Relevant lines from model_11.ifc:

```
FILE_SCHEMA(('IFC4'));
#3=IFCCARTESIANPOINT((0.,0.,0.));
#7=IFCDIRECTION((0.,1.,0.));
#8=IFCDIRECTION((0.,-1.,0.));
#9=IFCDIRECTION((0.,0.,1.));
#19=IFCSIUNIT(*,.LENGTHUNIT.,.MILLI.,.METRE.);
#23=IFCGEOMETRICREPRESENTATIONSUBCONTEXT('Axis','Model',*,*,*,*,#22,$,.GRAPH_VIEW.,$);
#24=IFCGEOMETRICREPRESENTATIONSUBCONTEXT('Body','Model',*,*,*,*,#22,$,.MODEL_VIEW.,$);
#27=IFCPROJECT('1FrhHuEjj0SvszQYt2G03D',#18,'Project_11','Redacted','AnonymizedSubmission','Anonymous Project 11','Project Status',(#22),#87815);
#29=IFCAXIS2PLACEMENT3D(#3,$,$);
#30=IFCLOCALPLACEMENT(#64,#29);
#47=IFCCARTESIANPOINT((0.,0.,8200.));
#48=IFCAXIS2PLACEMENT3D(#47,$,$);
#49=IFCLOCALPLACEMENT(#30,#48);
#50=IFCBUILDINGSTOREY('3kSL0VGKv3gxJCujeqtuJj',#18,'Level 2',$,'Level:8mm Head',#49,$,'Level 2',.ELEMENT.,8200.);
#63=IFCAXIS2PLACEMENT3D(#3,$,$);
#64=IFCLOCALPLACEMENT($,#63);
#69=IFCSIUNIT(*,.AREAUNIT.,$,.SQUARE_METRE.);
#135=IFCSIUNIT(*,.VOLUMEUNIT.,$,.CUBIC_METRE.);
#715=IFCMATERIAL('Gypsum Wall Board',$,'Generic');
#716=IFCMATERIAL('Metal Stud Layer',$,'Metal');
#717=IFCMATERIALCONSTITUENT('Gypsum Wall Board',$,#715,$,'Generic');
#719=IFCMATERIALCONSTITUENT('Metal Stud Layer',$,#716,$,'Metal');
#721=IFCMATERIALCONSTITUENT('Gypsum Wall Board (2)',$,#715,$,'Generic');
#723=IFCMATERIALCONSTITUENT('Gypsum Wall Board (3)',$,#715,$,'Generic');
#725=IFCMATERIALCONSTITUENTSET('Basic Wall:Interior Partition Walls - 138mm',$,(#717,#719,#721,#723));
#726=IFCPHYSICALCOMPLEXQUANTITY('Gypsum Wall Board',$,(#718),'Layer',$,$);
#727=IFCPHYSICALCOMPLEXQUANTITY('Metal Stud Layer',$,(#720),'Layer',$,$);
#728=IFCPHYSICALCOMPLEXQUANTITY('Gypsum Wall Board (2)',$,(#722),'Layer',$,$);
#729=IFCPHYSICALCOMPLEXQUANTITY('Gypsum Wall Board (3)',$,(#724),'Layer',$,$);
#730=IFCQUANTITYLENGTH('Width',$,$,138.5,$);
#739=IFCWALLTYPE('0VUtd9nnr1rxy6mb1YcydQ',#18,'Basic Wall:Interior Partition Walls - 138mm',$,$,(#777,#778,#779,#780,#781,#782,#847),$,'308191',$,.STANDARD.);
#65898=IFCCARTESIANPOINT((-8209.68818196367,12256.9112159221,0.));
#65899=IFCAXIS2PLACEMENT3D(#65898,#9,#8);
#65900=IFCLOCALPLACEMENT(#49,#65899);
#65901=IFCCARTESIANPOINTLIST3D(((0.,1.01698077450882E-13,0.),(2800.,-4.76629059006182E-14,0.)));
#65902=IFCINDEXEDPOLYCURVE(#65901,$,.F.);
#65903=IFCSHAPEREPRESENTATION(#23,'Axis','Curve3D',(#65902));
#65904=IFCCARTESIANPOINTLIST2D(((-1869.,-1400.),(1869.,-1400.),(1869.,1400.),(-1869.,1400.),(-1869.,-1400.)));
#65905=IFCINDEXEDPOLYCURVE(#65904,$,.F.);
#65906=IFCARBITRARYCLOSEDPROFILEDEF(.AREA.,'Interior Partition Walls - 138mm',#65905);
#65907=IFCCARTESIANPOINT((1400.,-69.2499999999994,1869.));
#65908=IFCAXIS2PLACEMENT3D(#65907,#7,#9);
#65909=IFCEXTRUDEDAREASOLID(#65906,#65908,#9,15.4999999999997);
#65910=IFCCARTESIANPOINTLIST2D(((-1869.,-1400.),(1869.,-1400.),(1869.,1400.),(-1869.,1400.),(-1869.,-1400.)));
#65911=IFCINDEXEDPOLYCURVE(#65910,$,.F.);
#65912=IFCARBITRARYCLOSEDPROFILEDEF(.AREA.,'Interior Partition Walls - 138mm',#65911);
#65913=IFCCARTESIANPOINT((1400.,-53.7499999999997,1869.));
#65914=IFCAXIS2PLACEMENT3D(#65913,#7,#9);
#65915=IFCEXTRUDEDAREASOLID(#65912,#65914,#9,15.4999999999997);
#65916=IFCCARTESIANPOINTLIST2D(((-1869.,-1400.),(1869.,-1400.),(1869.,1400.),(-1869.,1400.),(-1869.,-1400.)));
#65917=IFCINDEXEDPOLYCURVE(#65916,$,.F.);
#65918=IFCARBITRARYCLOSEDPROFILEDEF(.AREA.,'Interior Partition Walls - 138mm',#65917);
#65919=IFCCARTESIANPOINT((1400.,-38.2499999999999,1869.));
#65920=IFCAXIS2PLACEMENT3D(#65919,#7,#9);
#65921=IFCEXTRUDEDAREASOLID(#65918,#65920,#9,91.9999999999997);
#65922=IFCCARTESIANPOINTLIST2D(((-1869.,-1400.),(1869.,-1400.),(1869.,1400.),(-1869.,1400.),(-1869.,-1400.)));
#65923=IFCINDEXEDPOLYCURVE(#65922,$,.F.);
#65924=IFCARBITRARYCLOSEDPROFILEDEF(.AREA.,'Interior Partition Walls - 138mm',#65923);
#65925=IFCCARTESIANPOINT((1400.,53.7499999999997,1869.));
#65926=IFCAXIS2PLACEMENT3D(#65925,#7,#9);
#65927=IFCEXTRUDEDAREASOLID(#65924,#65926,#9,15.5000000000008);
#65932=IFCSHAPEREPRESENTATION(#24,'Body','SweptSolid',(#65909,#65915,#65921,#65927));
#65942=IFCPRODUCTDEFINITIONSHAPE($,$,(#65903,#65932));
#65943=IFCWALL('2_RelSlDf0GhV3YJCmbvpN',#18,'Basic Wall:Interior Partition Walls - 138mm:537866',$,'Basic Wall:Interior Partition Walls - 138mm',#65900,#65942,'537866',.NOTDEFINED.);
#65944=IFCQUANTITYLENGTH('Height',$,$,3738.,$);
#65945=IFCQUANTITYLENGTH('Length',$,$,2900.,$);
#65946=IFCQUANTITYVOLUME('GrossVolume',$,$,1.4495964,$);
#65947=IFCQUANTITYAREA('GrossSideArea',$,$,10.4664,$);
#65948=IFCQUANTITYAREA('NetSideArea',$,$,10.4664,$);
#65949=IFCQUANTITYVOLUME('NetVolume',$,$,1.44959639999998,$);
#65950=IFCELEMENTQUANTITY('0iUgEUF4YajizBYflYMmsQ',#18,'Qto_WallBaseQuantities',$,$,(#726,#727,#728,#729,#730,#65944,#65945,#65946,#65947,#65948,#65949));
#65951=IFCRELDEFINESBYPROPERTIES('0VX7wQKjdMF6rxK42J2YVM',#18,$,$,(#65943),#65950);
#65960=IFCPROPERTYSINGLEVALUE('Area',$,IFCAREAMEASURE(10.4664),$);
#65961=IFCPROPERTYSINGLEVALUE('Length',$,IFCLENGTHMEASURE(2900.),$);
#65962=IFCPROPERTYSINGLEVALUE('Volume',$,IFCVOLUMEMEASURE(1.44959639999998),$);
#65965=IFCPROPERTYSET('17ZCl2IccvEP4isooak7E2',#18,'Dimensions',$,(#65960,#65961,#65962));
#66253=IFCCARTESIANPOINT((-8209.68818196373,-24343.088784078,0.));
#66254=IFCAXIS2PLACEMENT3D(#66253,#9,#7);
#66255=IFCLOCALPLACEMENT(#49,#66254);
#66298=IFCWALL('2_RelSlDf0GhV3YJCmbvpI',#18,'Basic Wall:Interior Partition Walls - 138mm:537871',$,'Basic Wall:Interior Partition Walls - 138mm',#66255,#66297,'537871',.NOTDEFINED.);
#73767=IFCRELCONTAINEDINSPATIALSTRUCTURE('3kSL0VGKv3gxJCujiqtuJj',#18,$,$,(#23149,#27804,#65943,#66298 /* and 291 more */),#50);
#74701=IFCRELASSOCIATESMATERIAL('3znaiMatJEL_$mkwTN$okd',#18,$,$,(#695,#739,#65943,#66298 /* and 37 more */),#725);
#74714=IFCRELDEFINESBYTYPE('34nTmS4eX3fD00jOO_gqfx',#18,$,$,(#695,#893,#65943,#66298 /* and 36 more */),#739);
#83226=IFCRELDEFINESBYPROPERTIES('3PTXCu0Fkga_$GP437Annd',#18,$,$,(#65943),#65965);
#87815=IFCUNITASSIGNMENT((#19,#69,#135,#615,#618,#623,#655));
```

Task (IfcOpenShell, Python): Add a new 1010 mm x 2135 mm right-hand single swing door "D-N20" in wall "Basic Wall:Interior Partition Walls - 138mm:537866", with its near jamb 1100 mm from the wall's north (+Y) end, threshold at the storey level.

```python
import numpy as np
import ifcopenshell
import ifcopenshell.api.feature
import ifcopenshell.api.geometry
import ifcopenshell.api.pset
import ifcopenshell.api.root
import ifcopenshell.api.spatial
import ifcopenshell.geom
import ifcopenshell.util.element
import ifcopenshell.util.placement
import ifcopenshell.util.representation
import ifcopenshell.util.shape
import ifcopenshell.util.unit

model = ifcopenshell.open("model_11.ifc")
unit_scale = ifcopenshell.util.unit.calculate_unit_scale(model)
area_scale = ifcopenshell.util.unit.calculate_unit_scale(model, "AREAUNIT")
volume_scale = ifcopenshell.util.unit.calculate_unit_scale(model, "VOLUMEUNIT")
settings = ifcopenshell.geom.settings()


def volume(element):
    """Net volume in cubic metres, openings subtracted."""
    shape = ifcopenshell.geom.create_shape(settings, element)
    return ifcopenshell.util.shape.get_volume(shape.geometry)


wall = model.by_guid("2_RelSlDf0GhV3YJCmbvpN")
storey = ifcopenshell.util.element.get_container(wall, ifc_class="IfcBuildingStorey")
context = ifcopenshell.util.representation.get_context(model, "Model", "Body", "MODEL_VIEW")
before = volume(wall)

width, height, from_end, sill = 1.01, 2.135, 1.1, 0.0  # metres

# The wall runs along its own X axis, and the end named is its -X end.
wall_shape = ifcopenshell.geom.create_shape(settings, wall)
x, y, z = ifcopenshell.util.shape.get_vertices(wall_shape.geometry).T
start = x.min() + from_end
face, thickness = float(y.min()), float(y.max() - y.min())
wall_matrix = ifcopenshell.util.placement.get_local_placement(wall.ObjectPlacement)
level = ifcopenshell.util.placement.get_local_placement(storey.ObjectPlacement)[2, 3]


def in_wall(x, y):
    """Placement at x, y metres in the wall's axes, at sill height."""
    matrix = wall_matrix.copy()
    matrix[:, 3] = wall_matrix @ np.array([x / unit_scale, y / unit_scale, 0.0, 1.0])
    matrix[2, 3] = level + sill / unit_scale
    return matrix


# Opening: a box that overshoots both wall faces by 50 mm.
opening = ifcopenshell.api.root.create_entity(model, ifc_class="IfcOpeningElement", predefined_type="OPENING")
box = ifcopenshell.api.geometry.add_wall_representation(
    model, context=context, length=width, height=height, thickness=thickness + 0.1
)
ifcopenshell.api.geometry.assign_representation(model, product=opening, representation=box)
ifcopenshell.api.geometry.edit_object_placement(model, product=opening, matrix=in_wall(start, face - 0.05), is_si=False)
ifcopenshell.api.feature.add_feature(model, feature=opening, element=wall)

door = ifcopenshell.api.root.create_entity(model, ifc_class="IfcDoor", name="D-N20", predefined_type="DOOR")
door.OverallWidth, door.OverallHeight = width / unit_scale, height / unit_scale
door.OperationType = "SINGLE_SWING_RIGHT"
body = ifcopenshell.api.geometry.add_door_representation(
    model,
    context=context,
    overall_width=door.OverallWidth,
    overall_height=door.OverallHeight,
    operation_type="SINGLE_SWING_RIGHT",
    lining_properties={"LiningDepth": thickness / unit_scale, "ThresholdDepth": thickness / unit_scale},
)
ifcopenshell.api.geometry.assign_representation(model, product=door, representation=body)
ifcopenshell.api.spatial.assign_container(model, products=[door], relating_structure=storey)
ifcopenshell.api.feature.add_filling(model, opening=opening, element=door)

# The lining spans the wall, so the door starts at the wall face.
ifcopenshell.api.geometry.edit_object_placement(model, product=door, matrix=in_wall(start, face), is_si=False)

after = volume(wall)

# Update the wall's stored quantities.
qto = model.by_id(ifcopenshell.util.element.get_pset(wall, "Qto_WallBaseQuantities", should_inherit=False)["id"])
ifcopenshell.api.pset.edit_qto(model, qto=qto, properties={
    "NetSideArea": after / thickness / area_scale,
    "NetVolume": after / volume_scale,
})
pset = model.by_id(ifcopenshell.util.element.get_pset(wall, "Dimensions", should_inherit=False)["id"])
ifcopenshell.api.pset.edit_pset(model, pset=pset, properties={
    "Area": model.create_entity("IfcAreaMeasure", after / thickness / area_scale),
    "Volume": model.create_entity("IfcVolumeMeasure", after / volume_scale),
})

print(f"wall volume {before:.3f} -> {after:.3f} m3")

model.write("model_11_edited.ifc")
```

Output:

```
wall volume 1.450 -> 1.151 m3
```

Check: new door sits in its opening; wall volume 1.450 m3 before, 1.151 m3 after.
